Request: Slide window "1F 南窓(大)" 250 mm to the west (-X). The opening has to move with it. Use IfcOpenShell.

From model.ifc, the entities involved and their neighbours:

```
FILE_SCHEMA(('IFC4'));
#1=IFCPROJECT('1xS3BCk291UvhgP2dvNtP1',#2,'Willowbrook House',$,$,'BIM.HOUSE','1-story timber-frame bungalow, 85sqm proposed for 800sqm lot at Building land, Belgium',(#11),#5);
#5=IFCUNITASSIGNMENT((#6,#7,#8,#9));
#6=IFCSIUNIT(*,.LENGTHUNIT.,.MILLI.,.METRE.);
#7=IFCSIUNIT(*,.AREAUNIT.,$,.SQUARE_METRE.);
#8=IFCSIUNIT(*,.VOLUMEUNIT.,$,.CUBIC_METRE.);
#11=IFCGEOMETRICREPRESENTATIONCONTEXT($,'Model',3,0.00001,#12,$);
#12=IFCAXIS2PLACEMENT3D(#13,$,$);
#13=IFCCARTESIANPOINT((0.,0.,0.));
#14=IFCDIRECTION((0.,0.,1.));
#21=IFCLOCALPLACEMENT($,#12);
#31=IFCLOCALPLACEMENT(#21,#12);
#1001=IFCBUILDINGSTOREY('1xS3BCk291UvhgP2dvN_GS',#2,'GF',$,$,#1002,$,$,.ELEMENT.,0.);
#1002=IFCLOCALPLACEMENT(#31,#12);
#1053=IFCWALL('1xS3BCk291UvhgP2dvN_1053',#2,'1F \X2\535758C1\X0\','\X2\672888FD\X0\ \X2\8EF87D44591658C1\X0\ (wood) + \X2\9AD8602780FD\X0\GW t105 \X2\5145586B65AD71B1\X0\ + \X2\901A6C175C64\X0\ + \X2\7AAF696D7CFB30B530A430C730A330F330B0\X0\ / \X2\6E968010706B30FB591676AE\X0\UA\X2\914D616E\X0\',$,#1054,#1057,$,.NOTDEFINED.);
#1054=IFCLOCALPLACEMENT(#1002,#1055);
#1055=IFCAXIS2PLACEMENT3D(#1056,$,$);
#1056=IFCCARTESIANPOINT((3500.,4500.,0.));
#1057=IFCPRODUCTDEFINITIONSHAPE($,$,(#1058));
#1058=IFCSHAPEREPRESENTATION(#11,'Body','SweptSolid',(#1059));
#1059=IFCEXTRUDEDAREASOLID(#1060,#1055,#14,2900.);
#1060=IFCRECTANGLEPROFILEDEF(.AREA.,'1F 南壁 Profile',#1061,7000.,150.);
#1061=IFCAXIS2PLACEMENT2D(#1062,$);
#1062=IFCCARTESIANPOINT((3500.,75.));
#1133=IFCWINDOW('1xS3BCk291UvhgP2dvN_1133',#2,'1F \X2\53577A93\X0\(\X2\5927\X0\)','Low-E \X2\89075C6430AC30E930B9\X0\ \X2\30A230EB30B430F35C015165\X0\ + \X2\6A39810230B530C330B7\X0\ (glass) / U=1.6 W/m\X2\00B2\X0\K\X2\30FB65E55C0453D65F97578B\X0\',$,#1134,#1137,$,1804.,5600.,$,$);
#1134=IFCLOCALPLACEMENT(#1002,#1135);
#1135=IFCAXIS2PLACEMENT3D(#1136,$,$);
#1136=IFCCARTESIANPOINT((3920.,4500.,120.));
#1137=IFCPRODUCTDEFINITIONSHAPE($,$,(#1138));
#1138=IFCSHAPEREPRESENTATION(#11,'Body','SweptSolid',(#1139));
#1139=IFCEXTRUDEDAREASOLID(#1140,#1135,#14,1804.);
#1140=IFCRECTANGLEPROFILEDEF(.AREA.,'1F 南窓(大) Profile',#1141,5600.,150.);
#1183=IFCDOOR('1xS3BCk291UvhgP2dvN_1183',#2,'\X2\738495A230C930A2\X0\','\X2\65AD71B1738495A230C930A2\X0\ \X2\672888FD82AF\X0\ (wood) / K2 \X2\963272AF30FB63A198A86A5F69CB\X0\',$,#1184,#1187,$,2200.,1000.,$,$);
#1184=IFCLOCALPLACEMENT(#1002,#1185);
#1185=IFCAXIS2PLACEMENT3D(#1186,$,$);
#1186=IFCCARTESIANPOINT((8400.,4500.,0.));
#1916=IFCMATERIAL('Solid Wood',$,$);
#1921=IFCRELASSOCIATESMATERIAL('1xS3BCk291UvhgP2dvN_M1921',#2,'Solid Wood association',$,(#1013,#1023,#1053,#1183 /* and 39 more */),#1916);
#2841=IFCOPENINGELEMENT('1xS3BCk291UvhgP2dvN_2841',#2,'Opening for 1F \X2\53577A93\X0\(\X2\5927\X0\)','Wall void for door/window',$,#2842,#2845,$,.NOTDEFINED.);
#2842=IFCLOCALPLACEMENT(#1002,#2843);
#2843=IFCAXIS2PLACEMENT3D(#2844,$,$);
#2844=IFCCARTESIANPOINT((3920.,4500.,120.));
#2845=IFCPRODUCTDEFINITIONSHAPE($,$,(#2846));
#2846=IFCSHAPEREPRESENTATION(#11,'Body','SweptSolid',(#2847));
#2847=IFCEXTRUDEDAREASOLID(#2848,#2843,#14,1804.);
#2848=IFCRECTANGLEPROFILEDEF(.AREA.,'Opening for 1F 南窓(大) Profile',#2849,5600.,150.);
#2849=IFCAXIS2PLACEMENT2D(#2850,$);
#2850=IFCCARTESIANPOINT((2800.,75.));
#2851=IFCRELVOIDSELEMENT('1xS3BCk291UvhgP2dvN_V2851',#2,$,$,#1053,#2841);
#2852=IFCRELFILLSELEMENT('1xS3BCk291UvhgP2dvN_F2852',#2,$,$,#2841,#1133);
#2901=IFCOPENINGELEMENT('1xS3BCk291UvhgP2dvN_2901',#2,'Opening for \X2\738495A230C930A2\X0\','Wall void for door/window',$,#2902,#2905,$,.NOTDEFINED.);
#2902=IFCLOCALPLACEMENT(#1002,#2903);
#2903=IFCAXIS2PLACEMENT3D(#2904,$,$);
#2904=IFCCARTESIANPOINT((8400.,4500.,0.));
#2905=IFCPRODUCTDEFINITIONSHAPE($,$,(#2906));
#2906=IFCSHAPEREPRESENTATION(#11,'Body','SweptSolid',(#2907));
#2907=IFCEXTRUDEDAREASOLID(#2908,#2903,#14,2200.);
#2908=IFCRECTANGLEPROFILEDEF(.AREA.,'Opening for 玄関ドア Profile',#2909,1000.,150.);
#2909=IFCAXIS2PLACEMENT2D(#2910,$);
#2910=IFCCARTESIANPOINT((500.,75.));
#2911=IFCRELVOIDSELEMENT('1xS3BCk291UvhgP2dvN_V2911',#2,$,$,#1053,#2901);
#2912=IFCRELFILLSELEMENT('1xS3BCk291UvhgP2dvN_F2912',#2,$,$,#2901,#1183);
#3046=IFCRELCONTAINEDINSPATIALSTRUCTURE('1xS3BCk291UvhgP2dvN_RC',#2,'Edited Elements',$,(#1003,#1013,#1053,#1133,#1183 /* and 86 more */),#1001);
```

```python
import ifcopenshell
import ifcopenshell.api.geometry
import ifcopenshell.util.placement

model = ifcopenshell.open("model.ifc")

window = model.by_id(1133)
opening = window.FillsVoids[0].RelatingOpeningElement
wall = opening.VoidsElements[0].RelatingBuildingElement

wall_matrix = ifcopenshell.util.placement.get_local_placement(wall.ObjectPlacement)
shift = wall_matrix[:3, 0] * -250.0
before = ifcopenshell.util.placement.get_local_placement(window.ObjectPlacement)[:3, 3].copy()

# The window is not placed relative to its opening, so move both.
for product in (opening, window):
    matrix = ifcopenshell.util.placement.get_local_placement(product.ObjectPlacement)
    matrix[:3, 3] += shift
    ifcopenshell.api.geometry.edit_object_placement(model, product=product, matrix=matrix, is_si=False)

after = ifcopenshell.util.placement.get_local_placement(window.ObjectPlacement)[:3, 3]
print("window moved by", (after - before).round(3) + 0.0)

model.write("model_edited.ifc")
```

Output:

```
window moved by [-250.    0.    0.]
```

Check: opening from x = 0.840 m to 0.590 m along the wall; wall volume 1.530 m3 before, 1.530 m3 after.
